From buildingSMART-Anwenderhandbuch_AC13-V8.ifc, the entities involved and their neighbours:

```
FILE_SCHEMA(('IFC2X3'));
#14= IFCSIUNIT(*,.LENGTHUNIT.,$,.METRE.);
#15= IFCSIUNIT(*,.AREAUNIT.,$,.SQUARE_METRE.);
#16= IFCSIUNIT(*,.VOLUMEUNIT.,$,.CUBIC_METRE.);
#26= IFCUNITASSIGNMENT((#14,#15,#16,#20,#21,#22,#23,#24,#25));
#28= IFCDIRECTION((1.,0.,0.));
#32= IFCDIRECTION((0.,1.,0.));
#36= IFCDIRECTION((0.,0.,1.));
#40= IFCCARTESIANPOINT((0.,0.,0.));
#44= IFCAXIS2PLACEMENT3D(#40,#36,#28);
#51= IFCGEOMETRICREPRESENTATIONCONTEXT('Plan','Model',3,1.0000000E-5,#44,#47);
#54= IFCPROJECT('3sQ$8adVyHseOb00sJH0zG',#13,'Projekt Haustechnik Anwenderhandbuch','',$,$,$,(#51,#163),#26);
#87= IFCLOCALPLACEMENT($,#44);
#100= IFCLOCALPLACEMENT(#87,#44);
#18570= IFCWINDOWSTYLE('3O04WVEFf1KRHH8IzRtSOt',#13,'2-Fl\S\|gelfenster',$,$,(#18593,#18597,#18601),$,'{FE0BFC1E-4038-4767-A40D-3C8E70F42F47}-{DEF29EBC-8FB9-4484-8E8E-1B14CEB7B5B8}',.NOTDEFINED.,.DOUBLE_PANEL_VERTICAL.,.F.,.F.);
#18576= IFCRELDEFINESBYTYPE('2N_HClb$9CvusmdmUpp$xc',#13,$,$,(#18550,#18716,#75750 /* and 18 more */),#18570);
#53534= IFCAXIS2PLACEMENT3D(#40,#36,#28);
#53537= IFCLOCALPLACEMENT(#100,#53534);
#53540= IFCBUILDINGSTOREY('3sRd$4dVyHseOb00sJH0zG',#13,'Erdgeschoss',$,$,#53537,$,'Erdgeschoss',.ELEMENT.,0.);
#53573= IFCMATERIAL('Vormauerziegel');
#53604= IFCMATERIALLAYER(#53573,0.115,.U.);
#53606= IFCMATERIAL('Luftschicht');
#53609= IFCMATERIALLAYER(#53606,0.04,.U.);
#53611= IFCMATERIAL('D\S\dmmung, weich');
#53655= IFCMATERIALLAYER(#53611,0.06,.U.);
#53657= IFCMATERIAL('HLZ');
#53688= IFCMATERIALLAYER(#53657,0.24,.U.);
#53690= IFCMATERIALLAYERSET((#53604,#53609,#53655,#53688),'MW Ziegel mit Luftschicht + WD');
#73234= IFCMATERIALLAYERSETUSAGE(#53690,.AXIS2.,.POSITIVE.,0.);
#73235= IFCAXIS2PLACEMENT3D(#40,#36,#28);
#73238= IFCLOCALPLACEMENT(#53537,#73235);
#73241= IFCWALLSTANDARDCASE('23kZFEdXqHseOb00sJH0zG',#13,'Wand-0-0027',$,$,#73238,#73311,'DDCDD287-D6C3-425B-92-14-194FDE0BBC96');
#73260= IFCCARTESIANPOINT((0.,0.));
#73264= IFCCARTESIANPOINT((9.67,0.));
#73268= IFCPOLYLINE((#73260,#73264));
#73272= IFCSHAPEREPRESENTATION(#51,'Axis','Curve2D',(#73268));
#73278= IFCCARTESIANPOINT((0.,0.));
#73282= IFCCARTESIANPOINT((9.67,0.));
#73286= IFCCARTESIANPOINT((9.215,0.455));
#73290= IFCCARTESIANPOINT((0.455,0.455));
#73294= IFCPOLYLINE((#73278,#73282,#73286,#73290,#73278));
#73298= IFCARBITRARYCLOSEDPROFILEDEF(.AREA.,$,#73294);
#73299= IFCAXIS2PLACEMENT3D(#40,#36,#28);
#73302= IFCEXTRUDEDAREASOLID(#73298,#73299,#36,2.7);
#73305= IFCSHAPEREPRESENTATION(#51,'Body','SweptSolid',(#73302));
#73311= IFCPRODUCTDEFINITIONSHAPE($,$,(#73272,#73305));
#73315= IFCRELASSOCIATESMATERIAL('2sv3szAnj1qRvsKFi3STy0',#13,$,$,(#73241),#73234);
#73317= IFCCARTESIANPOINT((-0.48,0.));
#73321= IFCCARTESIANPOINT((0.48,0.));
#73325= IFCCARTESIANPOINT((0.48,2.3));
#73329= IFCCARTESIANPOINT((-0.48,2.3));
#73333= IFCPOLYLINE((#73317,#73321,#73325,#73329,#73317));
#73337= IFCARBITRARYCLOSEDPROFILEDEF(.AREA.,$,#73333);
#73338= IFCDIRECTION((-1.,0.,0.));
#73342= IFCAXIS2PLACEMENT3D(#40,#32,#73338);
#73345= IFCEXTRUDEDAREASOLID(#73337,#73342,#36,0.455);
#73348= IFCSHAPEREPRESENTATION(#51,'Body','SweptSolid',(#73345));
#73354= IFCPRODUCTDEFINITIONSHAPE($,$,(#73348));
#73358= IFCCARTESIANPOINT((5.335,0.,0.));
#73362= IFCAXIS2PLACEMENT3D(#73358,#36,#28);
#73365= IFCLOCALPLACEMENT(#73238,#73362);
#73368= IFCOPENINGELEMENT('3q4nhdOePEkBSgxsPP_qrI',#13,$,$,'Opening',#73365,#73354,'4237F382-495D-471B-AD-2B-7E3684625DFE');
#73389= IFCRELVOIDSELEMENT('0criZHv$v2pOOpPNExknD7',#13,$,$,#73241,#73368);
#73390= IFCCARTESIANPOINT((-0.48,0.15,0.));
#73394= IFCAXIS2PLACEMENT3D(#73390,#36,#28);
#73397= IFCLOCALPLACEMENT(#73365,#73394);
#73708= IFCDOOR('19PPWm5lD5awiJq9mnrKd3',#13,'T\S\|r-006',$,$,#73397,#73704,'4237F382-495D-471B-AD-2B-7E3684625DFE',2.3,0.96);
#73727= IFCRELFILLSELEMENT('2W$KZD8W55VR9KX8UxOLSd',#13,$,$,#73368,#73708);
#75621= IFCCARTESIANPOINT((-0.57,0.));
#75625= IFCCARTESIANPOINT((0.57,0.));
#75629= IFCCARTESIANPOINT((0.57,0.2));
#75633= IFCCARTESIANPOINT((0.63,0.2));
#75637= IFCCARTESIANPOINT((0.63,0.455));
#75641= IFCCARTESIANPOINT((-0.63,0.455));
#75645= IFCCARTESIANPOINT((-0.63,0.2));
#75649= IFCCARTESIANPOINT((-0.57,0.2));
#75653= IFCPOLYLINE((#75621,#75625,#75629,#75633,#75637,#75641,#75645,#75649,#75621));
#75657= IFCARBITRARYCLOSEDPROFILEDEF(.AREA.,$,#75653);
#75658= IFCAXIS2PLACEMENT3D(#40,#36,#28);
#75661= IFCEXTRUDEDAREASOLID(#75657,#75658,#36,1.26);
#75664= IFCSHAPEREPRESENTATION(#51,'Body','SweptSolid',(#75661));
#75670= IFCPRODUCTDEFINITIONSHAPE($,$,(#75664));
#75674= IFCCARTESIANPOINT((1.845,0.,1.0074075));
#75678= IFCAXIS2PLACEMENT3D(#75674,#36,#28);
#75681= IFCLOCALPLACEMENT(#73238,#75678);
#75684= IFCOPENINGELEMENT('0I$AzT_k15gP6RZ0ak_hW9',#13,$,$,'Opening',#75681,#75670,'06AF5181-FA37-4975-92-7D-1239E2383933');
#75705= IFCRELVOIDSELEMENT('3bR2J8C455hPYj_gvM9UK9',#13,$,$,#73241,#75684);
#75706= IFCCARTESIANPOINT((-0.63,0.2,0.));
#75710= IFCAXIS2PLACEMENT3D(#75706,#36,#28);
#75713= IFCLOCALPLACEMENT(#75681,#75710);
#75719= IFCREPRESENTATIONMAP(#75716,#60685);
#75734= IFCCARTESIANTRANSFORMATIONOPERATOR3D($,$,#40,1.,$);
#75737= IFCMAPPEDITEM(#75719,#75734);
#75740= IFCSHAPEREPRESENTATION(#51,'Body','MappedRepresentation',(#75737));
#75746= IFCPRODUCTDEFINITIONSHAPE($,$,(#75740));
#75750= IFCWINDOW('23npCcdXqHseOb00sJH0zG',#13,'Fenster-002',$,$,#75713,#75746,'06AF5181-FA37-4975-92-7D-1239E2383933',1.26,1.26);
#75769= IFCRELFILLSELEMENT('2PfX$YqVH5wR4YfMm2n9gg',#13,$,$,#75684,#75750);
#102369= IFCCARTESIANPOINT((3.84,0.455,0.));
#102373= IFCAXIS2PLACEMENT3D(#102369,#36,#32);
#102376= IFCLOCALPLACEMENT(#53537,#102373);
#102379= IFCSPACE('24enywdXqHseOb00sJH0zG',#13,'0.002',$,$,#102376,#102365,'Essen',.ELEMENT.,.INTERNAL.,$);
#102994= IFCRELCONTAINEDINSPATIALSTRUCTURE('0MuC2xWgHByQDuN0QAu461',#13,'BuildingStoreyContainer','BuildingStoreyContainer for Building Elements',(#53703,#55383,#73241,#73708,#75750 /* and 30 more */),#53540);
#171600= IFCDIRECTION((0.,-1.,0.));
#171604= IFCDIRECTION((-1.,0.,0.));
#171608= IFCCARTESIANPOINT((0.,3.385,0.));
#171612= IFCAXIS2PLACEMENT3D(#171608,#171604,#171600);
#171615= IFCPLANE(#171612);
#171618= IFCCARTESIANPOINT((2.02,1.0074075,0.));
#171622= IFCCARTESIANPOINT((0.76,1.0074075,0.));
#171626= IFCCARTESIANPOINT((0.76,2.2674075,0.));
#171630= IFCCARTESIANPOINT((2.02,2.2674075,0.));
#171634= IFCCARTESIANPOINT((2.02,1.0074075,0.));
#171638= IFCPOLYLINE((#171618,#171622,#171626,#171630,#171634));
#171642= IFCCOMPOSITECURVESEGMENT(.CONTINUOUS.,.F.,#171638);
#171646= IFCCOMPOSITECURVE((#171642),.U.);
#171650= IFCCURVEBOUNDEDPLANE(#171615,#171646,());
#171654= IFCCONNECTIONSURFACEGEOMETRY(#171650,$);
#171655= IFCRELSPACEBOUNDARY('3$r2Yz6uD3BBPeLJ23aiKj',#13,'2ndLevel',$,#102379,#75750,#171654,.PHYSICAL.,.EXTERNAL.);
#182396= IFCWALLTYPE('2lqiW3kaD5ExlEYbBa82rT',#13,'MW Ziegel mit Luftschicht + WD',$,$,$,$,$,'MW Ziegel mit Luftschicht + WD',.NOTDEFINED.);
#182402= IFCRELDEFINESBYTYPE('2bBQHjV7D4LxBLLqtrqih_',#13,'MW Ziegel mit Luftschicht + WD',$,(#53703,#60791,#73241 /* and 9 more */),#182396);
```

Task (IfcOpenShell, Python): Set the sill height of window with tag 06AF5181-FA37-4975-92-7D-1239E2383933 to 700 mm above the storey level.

```python
import numpy as np
import ifcopenshell
import ifcopenshell.api.geometry
import ifcopenshell.geom
import ifcopenshell.util.element
import ifcopenshell.util.placement
import ifcopenshell.util.shape
import ifcopenshell.util.unit

model = ifcopenshell.open("buildingSMART-Anwenderhandbuch_AC13-V8.ifc")
unit_scale = ifcopenshell.util.unit.calculate_unit_scale(model)

window = model.by_guid("23npCcdXqHseOb00sJH0zG")
opening = window.FillsVoids[0].RelatingOpeningElement
storey = ifcopenshell.util.element.get_container(window, ifc_class="IfcBuildingStorey")
level = ifcopenshell.util.placement.get_local_placement(storey.ObjectPlacement)[2, 3]

# The opening's origin need not be at the sill, so measure its lowest point.
shape = ifcopenshell.geom.create_shape(ifcopenshell.geom.settings(), opening)
bottom = ifcopenshell.util.shape.get_shape_bottom_elevation(shape, shape.geometry) / unit_scale
dz = level + 0.7 / unit_scale - bottom

shift = np.array([0.0, 0.0, dz])
# The window is placed relative to its opening, so it follows when the opening moves.
matrix = ifcopenshell.util.placement.get_local_placement(opening.ObjectPlacement)
matrix[:3, 3] += shift
ifcopenshell.api.geometry.edit_object_placement(
    model, product=opening, matrix=matrix, is_si=False, should_transform_children=True
)

# Space boundary surfaces are stored in each space's coordinates; move them too.
for rel in window.ProvidesBoundaries:
    if not rel.ConnectionGeometry:
        continue
    surface = rel.ConnectionGeometry.SurfaceOnRelatingElement.BasisSurface
    space_matrix = ifcopenshell.util.placement.get_local_placement(rel.RelatingSpace.ObjectPlacement)
    point = np.array(surface.Position.Location.Coordinates) + space_matrix[:3, :3].T @ shift
    surface.Position = model.createIfcAxis2Placement3D(
        model.createIfcCartesianPoint(point.tolist()), surface.Position.Axis, surface.Position.RefDirection
    )

print(f"moved by {dz * unit_scale:+.3f} m")

model.write("buildingSMART-Anwenderhandbuch_AC13-V8_rev.ifc")
```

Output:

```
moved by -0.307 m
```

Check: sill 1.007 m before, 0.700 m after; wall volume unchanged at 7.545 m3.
